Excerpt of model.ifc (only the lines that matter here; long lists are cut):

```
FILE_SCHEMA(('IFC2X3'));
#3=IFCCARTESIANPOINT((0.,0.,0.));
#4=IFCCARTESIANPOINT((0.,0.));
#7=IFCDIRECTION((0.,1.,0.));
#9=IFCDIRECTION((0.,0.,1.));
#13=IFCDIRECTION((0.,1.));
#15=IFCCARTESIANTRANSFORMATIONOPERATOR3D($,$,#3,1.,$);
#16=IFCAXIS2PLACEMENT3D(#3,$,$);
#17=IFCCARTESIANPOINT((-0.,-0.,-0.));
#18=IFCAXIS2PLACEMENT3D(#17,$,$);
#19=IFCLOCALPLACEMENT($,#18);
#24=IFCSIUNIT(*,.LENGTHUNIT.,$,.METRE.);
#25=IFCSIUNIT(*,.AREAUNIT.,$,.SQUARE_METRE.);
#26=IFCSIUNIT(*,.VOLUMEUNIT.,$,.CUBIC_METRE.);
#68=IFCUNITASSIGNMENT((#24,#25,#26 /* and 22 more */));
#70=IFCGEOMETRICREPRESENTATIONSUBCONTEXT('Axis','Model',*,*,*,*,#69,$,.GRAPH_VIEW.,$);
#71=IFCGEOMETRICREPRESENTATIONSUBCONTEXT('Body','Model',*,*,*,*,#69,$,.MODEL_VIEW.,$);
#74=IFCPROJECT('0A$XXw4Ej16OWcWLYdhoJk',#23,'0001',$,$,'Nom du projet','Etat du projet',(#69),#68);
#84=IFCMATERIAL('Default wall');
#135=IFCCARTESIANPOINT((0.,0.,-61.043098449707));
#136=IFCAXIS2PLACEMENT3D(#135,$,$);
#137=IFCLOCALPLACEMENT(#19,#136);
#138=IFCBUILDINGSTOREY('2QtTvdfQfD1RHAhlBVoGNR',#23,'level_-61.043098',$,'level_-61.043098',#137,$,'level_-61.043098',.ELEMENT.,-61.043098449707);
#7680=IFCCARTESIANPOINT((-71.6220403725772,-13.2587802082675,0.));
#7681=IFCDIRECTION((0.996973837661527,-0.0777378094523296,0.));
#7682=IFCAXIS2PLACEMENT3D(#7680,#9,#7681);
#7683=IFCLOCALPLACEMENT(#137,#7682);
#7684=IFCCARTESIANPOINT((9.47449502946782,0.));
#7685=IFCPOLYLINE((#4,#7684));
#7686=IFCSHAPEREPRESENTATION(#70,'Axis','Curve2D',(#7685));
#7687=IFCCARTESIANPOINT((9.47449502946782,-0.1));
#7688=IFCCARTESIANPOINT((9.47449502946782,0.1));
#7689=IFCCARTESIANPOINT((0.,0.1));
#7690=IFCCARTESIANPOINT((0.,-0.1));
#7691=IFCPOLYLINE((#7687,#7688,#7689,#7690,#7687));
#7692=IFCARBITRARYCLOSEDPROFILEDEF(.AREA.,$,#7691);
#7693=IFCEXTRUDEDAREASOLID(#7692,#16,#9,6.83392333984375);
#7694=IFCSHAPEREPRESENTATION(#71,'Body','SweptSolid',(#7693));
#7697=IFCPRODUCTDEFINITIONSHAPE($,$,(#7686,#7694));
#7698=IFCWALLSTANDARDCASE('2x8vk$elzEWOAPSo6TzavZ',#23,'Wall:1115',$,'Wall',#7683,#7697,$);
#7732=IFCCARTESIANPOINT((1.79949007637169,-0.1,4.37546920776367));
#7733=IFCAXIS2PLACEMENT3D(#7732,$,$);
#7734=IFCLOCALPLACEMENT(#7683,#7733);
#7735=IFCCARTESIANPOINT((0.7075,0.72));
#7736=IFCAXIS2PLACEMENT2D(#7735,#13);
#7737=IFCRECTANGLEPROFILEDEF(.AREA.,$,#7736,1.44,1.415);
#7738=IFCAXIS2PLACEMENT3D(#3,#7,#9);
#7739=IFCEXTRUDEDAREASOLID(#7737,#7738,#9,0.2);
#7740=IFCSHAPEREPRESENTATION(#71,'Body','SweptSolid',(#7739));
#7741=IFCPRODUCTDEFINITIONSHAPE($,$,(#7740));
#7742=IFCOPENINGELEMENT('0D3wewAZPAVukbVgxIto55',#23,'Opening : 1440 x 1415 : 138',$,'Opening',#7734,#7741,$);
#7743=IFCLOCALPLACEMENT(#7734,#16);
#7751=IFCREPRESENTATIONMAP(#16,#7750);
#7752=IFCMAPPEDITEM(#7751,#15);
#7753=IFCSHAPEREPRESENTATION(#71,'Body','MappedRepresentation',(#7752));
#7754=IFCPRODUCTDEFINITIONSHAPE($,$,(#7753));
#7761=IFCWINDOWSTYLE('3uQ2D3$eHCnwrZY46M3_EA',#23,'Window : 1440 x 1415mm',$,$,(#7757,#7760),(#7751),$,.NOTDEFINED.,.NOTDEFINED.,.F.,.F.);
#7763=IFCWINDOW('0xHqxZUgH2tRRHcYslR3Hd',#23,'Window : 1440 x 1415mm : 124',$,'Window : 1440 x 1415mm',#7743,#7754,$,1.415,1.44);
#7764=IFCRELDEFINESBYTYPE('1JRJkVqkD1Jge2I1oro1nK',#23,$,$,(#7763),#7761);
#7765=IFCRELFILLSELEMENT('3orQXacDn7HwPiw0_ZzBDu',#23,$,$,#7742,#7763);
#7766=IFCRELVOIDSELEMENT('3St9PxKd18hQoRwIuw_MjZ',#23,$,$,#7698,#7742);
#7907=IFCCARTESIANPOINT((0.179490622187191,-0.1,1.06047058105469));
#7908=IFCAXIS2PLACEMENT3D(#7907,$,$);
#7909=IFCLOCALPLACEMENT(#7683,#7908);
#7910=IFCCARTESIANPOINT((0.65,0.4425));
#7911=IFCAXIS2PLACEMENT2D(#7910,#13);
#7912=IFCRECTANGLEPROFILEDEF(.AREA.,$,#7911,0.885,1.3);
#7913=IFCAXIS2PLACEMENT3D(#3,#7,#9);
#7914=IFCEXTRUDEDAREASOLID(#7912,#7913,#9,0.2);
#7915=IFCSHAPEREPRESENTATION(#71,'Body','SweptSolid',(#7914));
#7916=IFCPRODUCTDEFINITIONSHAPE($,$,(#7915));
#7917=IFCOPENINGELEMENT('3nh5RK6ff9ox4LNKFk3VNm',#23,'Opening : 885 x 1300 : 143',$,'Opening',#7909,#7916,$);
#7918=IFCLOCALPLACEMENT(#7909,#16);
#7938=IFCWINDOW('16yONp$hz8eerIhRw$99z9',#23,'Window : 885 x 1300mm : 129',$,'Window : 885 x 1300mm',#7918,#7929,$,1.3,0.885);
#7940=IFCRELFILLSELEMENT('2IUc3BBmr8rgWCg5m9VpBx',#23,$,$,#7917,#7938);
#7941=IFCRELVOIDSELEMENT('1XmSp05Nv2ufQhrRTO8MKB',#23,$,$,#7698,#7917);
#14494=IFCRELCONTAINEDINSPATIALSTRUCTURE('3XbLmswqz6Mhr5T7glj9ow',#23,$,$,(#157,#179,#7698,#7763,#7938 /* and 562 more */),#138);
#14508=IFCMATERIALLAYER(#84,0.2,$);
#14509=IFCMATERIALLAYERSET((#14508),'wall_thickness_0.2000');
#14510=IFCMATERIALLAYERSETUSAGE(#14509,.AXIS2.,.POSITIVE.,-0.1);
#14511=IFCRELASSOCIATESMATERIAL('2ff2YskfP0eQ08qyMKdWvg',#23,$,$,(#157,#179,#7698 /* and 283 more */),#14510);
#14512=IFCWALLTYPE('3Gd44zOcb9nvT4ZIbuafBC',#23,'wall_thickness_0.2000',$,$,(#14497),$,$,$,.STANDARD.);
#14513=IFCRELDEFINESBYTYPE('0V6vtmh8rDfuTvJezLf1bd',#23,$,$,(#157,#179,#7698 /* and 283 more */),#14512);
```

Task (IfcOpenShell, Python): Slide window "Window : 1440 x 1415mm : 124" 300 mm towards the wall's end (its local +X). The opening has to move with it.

```python
import ifcopenshell
import ifcopenshell.api.geometry
import ifcopenshell.util.placement
import ifcopenshell.util.unit

model = ifcopenshell.open("model.ifc")
unit_scale = ifcopenshell.util.unit.calculate_unit_scale(model)

window = model.by_id(7763)
opening = window.FillsVoids[0].RelatingOpeningElement
wall = opening.VoidsElements[0].RelatingBuildingElement

wall_matrix = ifcopenshell.util.placement.get_local_placement(wall.ObjectPlacement)
shift = wall_matrix[:3, 0] * 0.3 / unit_scale
before = ifcopenshell.util.placement.get_local_placement(window.ObjectPlacement)[:3, 3].copy()

# The window is placed relative to its opening, so it follows when the opening moves.
matrix = ifcopenshell.util.placement.get_local_placement(opening.ObjectPlacement)
matrix[:3, 3] += shift
ifcopenshell.api.geometry.edit_object_placement(
    model, product=opening, matrix=matrix, is_si=False, should_transform_children=True
)

after = ifcopenshell.util.placement.get_local_placement(window.ObjectPlacement)[:3, 3]
print("window moved by", (after - before).round(3) + 0.0)

model.write("model-out.ifc")
```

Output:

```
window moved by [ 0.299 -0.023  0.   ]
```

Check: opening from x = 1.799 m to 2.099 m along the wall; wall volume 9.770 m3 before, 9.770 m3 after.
